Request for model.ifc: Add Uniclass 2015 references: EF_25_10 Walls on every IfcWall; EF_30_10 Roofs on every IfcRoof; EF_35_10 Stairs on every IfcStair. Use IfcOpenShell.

First a look at what the model holds.

```python
import ifcopenshell

model = ifcopenshell.open("model.ifc")
print(model.schema)
print("classifications:", [c.Name for c in model.by_type("IfcClassification")])
for ifc_class in ("IfcDoor", "IfcRoof", "IfcStair", "IfcWall", "IfcWindow"):
    print(ifc_class, len(model.by_type(ifc_class)))
```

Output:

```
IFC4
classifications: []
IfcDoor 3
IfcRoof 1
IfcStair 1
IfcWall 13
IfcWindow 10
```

```python
import ifcopenshell
import ifcopenshell.api.classification

model = ifcopenshell.open("model.ifc")

system = ifcopenshell.api.classification.add_classification(model, classification="Uniclass 2015")

codes = {
    "IfcWall": ("EF_25_10", "Walls"),
    "IfcRoof": ("EF_30_10", "Roofs"),
    "IfcStair": ("EF_35_10", "Stairs"),
}
for ifc_class, (code, name) in codes.items():
    products = model.by_type(ifc_class)
    ifcopenshell.api.classification.add_reference(
        model, products=products, classification=system, identification=code, name=name
    )
    print(code, len(products))

model.write("model_v2.ifc")
```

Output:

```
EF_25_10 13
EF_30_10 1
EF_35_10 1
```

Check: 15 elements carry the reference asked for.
